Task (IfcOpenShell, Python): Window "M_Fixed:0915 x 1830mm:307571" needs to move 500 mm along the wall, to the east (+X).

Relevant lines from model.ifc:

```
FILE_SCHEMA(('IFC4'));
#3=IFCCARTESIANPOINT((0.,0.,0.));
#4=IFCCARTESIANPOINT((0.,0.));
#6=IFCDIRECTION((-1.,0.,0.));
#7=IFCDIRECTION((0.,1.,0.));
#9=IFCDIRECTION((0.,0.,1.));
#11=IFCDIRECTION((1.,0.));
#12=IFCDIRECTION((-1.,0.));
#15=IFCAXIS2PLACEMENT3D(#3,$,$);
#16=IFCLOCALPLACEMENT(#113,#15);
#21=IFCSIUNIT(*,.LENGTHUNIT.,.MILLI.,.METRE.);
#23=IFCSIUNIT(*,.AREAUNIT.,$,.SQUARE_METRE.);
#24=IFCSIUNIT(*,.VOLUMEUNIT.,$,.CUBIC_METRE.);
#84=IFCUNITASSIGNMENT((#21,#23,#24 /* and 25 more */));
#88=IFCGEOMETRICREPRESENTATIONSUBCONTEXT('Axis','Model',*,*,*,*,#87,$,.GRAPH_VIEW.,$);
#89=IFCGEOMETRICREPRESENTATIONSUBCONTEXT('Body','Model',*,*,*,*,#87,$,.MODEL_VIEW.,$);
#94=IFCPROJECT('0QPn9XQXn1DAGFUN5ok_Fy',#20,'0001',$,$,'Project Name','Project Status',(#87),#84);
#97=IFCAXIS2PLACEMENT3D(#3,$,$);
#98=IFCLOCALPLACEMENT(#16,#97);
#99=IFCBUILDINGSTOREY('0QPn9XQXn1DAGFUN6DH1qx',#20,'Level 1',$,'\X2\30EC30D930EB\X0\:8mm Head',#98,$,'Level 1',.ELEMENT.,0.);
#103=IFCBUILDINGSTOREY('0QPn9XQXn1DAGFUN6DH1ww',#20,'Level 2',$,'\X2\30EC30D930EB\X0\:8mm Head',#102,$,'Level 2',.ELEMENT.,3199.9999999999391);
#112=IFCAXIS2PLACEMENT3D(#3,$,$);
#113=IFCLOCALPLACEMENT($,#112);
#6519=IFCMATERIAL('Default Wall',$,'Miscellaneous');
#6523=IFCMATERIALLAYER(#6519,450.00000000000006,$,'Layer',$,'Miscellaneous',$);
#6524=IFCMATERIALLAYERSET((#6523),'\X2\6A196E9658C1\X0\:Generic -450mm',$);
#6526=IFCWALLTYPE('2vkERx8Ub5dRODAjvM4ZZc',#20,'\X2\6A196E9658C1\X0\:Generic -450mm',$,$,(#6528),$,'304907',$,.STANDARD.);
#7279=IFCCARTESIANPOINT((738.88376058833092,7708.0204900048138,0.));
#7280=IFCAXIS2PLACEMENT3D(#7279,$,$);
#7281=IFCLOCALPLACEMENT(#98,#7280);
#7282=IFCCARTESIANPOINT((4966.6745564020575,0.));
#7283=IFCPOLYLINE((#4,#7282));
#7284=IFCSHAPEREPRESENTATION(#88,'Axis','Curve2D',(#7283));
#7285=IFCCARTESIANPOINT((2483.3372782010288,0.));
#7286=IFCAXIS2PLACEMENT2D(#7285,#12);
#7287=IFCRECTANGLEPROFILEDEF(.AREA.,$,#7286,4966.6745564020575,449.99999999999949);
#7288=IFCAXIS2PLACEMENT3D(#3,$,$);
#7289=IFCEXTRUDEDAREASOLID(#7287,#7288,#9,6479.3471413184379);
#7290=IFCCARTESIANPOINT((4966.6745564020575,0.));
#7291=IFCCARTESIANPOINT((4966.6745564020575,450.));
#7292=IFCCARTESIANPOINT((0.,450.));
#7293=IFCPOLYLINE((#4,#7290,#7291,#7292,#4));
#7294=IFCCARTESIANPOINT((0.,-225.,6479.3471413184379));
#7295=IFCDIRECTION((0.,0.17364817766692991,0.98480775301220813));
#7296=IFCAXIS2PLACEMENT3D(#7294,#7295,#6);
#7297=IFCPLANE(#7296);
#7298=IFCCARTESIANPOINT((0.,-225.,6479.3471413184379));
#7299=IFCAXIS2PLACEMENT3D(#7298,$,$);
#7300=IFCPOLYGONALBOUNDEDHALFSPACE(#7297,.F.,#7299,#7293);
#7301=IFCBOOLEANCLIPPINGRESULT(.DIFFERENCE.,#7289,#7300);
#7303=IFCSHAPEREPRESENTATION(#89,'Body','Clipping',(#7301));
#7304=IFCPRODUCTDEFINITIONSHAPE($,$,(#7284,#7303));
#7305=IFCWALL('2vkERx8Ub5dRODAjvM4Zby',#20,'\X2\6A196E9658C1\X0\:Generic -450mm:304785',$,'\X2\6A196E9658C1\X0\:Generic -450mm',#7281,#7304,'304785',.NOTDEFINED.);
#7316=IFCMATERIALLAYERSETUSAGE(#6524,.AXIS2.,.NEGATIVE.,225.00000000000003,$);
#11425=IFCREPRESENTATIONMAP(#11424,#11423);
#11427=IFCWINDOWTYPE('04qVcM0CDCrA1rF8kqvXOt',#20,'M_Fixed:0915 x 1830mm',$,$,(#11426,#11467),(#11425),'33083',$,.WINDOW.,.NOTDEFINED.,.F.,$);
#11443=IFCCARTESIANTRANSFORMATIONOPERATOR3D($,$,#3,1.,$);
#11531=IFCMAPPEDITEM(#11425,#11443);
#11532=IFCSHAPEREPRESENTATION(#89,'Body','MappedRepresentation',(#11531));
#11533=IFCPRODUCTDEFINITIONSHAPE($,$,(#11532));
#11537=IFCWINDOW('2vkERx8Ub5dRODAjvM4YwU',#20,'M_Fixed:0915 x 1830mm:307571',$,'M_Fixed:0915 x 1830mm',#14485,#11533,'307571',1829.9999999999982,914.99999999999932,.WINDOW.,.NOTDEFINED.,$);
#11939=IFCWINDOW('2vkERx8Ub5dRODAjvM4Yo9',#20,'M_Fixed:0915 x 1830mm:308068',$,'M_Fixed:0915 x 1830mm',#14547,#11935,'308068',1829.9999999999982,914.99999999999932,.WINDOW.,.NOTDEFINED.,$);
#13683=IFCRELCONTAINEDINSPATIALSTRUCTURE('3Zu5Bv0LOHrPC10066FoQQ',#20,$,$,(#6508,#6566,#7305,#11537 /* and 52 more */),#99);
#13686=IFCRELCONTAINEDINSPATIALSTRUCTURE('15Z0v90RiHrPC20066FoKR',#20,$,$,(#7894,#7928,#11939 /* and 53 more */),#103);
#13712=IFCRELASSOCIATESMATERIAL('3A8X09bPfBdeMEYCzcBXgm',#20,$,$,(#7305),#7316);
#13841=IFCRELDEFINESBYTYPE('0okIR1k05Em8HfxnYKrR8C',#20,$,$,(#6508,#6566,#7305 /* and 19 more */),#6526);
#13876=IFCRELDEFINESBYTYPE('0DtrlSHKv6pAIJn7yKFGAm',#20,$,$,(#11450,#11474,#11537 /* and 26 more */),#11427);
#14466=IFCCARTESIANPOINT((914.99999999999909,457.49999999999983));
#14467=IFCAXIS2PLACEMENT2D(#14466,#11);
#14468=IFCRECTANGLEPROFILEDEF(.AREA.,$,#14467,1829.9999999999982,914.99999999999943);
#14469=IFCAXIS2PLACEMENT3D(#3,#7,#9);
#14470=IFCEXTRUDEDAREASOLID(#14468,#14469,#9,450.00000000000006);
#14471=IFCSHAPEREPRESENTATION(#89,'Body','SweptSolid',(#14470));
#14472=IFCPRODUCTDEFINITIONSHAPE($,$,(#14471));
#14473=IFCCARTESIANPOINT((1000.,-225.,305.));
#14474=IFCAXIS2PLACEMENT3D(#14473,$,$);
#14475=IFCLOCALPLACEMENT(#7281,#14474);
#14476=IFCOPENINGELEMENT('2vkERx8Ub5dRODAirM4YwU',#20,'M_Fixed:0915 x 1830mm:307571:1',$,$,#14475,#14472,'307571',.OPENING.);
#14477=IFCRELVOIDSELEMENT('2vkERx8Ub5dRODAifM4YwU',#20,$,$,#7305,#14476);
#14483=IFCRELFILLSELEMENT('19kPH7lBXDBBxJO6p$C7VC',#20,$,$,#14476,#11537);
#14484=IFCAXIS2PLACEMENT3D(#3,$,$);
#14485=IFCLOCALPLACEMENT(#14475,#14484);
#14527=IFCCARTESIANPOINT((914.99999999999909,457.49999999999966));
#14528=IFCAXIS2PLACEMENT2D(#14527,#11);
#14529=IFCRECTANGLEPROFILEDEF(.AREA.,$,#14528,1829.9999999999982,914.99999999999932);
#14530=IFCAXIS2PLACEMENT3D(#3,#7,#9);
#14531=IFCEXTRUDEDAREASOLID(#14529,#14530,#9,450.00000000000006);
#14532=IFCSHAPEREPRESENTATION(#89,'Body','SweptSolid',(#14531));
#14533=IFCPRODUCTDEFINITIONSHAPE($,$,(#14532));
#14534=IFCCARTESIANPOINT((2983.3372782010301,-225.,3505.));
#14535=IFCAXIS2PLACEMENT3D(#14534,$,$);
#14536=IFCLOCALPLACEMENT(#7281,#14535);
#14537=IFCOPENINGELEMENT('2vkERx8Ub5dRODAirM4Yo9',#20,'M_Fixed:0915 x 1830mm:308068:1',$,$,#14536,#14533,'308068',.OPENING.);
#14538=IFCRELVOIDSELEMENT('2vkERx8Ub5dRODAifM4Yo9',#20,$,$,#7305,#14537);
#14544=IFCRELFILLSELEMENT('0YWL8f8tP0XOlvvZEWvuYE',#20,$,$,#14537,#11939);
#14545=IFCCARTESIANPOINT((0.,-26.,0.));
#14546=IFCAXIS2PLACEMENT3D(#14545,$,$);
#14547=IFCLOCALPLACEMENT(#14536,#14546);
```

```python
import ifcopenshell
import ifcopenshell.api.geometry
import ifcopenshell.util.placement
import ifcopenshell.util.unit

model = ifcopenshell.open("model.ifc")
unit_scale = ifcopenshell.util.unit.calculate_unit_scale(model)

window = model.by_guid("2vkERx8Ub5dRODAjvM4YwU")
opening = window.FillsVoids[0].RelatingOpeningElement
wall = opening.VoidsElements[0].RelatingBuildingElement

wall_matrix = ifcopenshell.util.placement.get_local_placement(wall.ObjectPlacement)
shift = wall_matrix[:3, 0] * 0.5 / unit_scale
before = ifcopenshell.util.placement.get_local_placement(window.ObjectPlacement)[:3, 3].copy()

# The window is placed relative to its opening, so it follows when the opening moves.
matrix = ifcopenshell.util.placement.get_local_placement(opening.ObjectPlacement)
matrix[:3, 3] += shift
ifcopenshell.api.geometry.edit_object_placement(
    model, product=opening, matrix=matrix, is_si=False, should_transform_children=True
)

after = ifcopenshell.util.placement.get_local_placement(window.ObjectPlacement)[:3, 3]
print("window moved by", (after - before).round(3) + 0.0)

model.write("model_updated.ifc")
```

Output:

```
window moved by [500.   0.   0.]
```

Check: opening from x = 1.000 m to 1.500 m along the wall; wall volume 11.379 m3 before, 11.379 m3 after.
